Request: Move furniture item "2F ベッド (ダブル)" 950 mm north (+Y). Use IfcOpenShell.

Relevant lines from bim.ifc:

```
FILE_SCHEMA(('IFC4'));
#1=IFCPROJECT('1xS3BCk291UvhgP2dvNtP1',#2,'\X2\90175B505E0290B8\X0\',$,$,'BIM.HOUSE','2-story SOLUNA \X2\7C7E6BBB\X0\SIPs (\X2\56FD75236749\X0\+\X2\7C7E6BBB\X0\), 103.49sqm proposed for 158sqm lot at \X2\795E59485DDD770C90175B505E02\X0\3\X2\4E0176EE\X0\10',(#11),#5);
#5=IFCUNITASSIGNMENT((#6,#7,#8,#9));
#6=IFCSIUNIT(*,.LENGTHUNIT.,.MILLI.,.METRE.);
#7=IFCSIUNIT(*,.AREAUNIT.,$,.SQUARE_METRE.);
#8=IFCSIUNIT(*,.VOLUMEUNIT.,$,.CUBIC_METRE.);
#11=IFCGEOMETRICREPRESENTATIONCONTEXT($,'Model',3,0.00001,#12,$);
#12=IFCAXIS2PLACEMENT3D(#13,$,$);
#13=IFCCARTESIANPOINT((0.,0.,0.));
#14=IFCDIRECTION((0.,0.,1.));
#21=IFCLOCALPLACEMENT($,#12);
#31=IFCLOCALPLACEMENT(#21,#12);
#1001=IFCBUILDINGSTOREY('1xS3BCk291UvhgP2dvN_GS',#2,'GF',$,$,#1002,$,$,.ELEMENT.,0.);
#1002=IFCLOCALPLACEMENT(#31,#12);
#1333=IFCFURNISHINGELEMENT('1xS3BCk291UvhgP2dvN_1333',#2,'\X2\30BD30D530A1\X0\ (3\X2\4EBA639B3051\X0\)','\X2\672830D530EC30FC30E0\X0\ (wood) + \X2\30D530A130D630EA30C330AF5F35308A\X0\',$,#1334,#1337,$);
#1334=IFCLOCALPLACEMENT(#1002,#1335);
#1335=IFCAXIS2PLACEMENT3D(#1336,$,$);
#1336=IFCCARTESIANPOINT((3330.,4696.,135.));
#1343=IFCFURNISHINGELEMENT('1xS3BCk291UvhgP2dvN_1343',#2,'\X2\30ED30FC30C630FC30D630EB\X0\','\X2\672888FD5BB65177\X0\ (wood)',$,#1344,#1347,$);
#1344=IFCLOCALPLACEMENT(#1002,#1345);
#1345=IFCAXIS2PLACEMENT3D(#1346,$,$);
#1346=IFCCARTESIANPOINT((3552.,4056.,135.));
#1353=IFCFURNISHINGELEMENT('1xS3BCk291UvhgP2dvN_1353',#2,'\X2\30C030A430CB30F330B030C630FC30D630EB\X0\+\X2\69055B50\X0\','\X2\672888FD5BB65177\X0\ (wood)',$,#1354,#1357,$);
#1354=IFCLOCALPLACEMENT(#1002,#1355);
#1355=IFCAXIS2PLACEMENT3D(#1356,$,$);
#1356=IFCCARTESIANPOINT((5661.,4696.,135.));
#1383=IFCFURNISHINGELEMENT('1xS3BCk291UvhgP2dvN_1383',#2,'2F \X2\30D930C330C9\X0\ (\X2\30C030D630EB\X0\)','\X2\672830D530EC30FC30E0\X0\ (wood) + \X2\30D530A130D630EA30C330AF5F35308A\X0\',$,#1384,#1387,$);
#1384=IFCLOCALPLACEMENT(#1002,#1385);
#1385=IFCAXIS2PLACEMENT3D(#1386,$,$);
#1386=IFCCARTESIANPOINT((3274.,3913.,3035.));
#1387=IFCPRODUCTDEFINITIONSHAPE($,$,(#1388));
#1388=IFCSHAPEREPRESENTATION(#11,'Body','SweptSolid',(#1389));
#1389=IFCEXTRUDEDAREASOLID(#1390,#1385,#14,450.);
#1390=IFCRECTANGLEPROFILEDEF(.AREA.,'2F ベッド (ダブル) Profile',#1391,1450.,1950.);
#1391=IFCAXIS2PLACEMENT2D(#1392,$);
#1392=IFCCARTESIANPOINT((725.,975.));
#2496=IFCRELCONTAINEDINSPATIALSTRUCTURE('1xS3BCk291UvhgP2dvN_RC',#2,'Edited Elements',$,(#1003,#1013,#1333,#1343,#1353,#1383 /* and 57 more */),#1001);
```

```python
import ifcopenshell
import ifcopenshell.api.geometry
import ifcopenshell.util.placement
import ifcopenshell.util.unit

model = ifcopenshell.open("bim.ifc")
unit_scale = ifcopenshell.util.unit.calculate_unit_scale(model)

item = model.by_guid("1xS3BCk291UvhgP2dvN_1383")
matrix = ifcopenshell.util.placement.get_local_placement(item.ObjectPlacement)
matrix[1, 3] += 0.95 / unit_scale
ifcopenshell.api.geometry.edit_object_placement(model, product=item, matrix=matrix, is_si=False)

print(ifcopenshell.util.placement.get_local_placement(item.ObjectPlacement).round(3) + 0.0)

model.write("bim_v2.ifc")
```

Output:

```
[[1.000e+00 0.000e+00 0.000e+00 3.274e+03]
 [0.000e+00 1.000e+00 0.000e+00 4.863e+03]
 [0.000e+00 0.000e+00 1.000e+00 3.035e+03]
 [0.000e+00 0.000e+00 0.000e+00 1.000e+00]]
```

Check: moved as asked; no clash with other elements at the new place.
